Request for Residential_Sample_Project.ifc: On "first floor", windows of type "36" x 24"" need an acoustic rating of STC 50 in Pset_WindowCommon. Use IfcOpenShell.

First a look at what the model holds.

```python
import ifcopenshell
import ifcopenshell.util.element

model = ifcopenshell.open("Residential_Sample_Project.ifc")
print(model.schema)
storey = next(s for s in model.by_type("IfcBuildingStorey") if s.Name == "first floor")
windows = [e for e in ifcopenshell.util.element.get_decomposition(storey) if e.is_a("IfcWindow")]
seen = {}
for e in windows:
    element_type = ifcopenshell.util.element.get_type(e)
    key = (element_type.Name if element_type != e and element_type else None, ifcopenshell.util.element.get_pset(e, "Pset_WindowCommon", "AcousticRating"))
    seen[key] = seen.get(key, 0) + 1
for (name, value), count in sorted(seen.items(), key=str):
    print(count, "x", name, "|", value)
```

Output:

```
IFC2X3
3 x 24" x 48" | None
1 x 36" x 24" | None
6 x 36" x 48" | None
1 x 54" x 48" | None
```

```python
import ifcopenshell
import ifcopenshell.api.pset
import ifcopenshell.util.element

model = ifcopenshell.open("Residential_Sample_Project.ifc")

storey = next(s for s in model.by_type("IfcBuildingStorey") if s.Name == "first floor")
windows = [e for e in ifcopenshell.util.element.get_decomposition(storey) if e.is_a("IfcWindow")]

count = 0
for e in windows:
    element_type = ifcopenshell.util.element.get_type(e)
    if element_type in (None, e) or element_type.Name != '36" x 24"':
        continue
    # add_pset returns the element's existing set when there is one.
    pset = ifcopenshell.api.pset.add_pset(model, product=e, name="Pset_WindowCommon")
    ifcopenshell.api.pset.edit_pset(model, pset=pset, properties={"AcousticRating": "STC 50"})
    count += 1

print(count, "windows updated")

model.write("Residential_Sample_Project_updated.ifc")
```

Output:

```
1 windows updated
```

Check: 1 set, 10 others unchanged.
